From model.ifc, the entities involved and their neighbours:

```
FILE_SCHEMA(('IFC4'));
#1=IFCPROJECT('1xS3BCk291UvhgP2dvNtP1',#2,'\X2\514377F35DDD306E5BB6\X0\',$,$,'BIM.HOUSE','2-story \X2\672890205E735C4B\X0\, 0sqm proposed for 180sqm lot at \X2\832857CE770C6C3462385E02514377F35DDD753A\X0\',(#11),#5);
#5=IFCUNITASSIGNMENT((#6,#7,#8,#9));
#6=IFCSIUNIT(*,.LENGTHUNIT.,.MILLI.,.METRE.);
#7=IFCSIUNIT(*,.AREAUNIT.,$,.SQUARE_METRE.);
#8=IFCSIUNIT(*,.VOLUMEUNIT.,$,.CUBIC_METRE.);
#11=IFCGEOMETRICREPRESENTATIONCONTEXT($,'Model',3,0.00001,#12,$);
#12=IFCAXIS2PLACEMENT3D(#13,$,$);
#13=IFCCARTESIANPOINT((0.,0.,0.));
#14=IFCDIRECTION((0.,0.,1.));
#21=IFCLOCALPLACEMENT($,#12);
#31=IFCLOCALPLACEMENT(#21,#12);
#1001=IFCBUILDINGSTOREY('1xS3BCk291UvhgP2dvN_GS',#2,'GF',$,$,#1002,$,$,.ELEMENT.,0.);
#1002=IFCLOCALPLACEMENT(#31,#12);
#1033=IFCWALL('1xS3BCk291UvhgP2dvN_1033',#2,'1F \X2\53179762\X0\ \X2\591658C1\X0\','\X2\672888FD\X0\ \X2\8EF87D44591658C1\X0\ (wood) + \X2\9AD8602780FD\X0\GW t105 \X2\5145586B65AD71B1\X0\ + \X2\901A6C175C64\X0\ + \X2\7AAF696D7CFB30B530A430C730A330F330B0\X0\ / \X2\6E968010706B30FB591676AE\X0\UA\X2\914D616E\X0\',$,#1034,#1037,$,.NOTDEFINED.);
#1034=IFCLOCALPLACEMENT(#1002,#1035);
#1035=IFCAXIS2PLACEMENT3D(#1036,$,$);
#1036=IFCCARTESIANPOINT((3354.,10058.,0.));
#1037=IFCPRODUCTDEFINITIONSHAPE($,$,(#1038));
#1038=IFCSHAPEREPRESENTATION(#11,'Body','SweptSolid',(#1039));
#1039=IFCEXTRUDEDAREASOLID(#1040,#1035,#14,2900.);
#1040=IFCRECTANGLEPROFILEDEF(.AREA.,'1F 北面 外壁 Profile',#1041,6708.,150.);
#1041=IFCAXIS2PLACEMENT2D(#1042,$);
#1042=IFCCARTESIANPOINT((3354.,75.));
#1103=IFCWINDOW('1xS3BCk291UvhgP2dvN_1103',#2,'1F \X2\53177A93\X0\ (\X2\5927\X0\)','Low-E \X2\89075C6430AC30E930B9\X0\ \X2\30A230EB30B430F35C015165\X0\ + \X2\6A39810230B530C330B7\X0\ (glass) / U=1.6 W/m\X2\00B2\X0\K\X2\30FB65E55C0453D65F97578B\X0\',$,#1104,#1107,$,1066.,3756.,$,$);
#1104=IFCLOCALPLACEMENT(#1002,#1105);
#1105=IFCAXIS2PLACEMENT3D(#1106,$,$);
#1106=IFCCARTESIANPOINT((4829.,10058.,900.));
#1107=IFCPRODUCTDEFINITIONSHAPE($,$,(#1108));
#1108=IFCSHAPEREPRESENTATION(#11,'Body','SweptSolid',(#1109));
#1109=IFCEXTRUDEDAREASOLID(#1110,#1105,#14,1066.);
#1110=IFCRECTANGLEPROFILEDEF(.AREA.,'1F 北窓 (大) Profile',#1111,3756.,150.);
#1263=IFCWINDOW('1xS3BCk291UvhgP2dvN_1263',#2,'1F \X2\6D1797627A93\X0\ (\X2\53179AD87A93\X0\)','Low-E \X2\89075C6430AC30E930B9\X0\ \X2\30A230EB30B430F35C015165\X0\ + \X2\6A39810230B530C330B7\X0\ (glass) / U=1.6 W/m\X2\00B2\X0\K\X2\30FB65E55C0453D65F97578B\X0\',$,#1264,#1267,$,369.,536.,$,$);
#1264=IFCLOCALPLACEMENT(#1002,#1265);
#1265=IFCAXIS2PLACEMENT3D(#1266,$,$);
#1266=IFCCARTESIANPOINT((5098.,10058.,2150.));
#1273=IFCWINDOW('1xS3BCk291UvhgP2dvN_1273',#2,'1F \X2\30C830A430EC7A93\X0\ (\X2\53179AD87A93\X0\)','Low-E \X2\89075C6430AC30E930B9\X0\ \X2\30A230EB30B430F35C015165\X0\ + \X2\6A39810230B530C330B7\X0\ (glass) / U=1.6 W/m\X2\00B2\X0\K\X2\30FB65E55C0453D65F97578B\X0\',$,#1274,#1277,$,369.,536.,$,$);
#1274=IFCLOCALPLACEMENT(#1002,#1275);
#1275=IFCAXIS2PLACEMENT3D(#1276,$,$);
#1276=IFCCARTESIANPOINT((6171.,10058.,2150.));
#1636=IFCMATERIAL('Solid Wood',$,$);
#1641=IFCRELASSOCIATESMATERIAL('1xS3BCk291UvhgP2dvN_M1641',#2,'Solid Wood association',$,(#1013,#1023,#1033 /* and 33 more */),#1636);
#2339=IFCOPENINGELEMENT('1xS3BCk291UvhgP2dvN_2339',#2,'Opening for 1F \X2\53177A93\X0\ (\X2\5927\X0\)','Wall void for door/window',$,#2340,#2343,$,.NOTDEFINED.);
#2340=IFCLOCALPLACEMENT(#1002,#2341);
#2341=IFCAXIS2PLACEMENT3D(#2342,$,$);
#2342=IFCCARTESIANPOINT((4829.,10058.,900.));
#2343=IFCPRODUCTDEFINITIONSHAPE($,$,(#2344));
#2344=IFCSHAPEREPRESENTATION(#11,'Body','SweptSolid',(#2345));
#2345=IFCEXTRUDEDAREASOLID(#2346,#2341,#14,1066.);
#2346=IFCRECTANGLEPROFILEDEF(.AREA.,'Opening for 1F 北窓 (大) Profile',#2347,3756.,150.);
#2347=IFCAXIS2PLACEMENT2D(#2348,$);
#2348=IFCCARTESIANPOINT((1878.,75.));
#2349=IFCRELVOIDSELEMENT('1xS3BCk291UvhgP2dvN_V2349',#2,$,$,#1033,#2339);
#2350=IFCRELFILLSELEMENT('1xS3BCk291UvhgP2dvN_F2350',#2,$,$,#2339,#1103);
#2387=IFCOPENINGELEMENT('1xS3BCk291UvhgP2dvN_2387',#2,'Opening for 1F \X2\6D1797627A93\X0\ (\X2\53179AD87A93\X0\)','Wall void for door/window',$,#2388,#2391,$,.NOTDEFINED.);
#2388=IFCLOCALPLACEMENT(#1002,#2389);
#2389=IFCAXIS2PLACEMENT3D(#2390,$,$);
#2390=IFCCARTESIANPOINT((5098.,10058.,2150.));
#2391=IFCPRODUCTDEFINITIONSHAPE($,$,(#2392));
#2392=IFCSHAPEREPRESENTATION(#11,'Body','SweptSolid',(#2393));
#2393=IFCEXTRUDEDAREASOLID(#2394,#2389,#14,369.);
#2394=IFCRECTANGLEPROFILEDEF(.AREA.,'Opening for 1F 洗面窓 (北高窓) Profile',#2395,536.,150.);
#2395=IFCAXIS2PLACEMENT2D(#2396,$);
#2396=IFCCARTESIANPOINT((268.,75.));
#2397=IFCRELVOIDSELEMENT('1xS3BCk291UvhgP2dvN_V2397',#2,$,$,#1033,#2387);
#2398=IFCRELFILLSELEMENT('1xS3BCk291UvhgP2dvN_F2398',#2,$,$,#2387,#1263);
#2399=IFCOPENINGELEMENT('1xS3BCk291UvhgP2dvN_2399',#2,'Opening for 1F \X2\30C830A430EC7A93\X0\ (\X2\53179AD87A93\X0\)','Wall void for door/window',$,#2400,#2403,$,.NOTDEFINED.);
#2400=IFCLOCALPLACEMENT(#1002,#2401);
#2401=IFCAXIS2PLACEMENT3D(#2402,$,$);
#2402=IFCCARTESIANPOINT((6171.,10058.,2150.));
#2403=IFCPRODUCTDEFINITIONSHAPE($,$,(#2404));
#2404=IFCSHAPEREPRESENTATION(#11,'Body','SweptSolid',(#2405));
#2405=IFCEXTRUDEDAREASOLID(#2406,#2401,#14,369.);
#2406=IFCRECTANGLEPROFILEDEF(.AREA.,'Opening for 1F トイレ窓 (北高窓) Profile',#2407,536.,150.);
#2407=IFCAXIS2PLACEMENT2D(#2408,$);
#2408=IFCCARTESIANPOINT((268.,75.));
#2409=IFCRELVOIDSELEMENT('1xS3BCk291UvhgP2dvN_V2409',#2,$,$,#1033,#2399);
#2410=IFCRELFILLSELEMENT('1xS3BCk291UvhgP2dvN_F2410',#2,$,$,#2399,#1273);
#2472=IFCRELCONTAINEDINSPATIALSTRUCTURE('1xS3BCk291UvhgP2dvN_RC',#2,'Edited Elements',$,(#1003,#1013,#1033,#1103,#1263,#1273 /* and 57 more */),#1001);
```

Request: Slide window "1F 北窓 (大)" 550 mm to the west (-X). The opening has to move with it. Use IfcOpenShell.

```python
import ifcopenshell
import ifcopenshell.api.geometry
import ifcopenshell.util.placement
import ifcopenshell.util.unit

model = ifcopenshell.open("model.ifc")
unit_scale = ifcopenshell.util.unit.calculate_unit_scale(model)

window = model.by_guid("1xS3BCk291UvhgP2dvN_1103")
opening = window.FillsVoids[0].RelatingOpeningElement
wall = opening.VoidsElements[0].RelatingBuildingElement

wall_matrix = ifcopenshell.util.placement.get_local_placement(wall.ObjectPlacement)
shift = wall_matrix[:3, 0] * -0.55 / unit_scale
before = ifcopenshell.util.placement.get_local_placement(window.ObjectPlacement)[:3, 3].copy()

# The window is not placed relative to its opening, so move both.
for product in (opening, window):
    matrix = ifcopenshell.util.placement.get_local_placement(product.ObjectPlacement)
    matrix[:3, 3] += shift
    ifcopenshell.api.geometry.edit_object_placement(model, product=product, matrix=matrix, is_si=False)

after = ifcopenshell.util.placement.get_local_placement(window.ObjectPlacement)[:3, 3]
print("window moved by", (after - before).round(3) + 0.0)

model.write("model_v2.ifc")
```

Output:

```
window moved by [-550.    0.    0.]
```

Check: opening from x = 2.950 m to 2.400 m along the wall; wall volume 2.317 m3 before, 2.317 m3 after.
